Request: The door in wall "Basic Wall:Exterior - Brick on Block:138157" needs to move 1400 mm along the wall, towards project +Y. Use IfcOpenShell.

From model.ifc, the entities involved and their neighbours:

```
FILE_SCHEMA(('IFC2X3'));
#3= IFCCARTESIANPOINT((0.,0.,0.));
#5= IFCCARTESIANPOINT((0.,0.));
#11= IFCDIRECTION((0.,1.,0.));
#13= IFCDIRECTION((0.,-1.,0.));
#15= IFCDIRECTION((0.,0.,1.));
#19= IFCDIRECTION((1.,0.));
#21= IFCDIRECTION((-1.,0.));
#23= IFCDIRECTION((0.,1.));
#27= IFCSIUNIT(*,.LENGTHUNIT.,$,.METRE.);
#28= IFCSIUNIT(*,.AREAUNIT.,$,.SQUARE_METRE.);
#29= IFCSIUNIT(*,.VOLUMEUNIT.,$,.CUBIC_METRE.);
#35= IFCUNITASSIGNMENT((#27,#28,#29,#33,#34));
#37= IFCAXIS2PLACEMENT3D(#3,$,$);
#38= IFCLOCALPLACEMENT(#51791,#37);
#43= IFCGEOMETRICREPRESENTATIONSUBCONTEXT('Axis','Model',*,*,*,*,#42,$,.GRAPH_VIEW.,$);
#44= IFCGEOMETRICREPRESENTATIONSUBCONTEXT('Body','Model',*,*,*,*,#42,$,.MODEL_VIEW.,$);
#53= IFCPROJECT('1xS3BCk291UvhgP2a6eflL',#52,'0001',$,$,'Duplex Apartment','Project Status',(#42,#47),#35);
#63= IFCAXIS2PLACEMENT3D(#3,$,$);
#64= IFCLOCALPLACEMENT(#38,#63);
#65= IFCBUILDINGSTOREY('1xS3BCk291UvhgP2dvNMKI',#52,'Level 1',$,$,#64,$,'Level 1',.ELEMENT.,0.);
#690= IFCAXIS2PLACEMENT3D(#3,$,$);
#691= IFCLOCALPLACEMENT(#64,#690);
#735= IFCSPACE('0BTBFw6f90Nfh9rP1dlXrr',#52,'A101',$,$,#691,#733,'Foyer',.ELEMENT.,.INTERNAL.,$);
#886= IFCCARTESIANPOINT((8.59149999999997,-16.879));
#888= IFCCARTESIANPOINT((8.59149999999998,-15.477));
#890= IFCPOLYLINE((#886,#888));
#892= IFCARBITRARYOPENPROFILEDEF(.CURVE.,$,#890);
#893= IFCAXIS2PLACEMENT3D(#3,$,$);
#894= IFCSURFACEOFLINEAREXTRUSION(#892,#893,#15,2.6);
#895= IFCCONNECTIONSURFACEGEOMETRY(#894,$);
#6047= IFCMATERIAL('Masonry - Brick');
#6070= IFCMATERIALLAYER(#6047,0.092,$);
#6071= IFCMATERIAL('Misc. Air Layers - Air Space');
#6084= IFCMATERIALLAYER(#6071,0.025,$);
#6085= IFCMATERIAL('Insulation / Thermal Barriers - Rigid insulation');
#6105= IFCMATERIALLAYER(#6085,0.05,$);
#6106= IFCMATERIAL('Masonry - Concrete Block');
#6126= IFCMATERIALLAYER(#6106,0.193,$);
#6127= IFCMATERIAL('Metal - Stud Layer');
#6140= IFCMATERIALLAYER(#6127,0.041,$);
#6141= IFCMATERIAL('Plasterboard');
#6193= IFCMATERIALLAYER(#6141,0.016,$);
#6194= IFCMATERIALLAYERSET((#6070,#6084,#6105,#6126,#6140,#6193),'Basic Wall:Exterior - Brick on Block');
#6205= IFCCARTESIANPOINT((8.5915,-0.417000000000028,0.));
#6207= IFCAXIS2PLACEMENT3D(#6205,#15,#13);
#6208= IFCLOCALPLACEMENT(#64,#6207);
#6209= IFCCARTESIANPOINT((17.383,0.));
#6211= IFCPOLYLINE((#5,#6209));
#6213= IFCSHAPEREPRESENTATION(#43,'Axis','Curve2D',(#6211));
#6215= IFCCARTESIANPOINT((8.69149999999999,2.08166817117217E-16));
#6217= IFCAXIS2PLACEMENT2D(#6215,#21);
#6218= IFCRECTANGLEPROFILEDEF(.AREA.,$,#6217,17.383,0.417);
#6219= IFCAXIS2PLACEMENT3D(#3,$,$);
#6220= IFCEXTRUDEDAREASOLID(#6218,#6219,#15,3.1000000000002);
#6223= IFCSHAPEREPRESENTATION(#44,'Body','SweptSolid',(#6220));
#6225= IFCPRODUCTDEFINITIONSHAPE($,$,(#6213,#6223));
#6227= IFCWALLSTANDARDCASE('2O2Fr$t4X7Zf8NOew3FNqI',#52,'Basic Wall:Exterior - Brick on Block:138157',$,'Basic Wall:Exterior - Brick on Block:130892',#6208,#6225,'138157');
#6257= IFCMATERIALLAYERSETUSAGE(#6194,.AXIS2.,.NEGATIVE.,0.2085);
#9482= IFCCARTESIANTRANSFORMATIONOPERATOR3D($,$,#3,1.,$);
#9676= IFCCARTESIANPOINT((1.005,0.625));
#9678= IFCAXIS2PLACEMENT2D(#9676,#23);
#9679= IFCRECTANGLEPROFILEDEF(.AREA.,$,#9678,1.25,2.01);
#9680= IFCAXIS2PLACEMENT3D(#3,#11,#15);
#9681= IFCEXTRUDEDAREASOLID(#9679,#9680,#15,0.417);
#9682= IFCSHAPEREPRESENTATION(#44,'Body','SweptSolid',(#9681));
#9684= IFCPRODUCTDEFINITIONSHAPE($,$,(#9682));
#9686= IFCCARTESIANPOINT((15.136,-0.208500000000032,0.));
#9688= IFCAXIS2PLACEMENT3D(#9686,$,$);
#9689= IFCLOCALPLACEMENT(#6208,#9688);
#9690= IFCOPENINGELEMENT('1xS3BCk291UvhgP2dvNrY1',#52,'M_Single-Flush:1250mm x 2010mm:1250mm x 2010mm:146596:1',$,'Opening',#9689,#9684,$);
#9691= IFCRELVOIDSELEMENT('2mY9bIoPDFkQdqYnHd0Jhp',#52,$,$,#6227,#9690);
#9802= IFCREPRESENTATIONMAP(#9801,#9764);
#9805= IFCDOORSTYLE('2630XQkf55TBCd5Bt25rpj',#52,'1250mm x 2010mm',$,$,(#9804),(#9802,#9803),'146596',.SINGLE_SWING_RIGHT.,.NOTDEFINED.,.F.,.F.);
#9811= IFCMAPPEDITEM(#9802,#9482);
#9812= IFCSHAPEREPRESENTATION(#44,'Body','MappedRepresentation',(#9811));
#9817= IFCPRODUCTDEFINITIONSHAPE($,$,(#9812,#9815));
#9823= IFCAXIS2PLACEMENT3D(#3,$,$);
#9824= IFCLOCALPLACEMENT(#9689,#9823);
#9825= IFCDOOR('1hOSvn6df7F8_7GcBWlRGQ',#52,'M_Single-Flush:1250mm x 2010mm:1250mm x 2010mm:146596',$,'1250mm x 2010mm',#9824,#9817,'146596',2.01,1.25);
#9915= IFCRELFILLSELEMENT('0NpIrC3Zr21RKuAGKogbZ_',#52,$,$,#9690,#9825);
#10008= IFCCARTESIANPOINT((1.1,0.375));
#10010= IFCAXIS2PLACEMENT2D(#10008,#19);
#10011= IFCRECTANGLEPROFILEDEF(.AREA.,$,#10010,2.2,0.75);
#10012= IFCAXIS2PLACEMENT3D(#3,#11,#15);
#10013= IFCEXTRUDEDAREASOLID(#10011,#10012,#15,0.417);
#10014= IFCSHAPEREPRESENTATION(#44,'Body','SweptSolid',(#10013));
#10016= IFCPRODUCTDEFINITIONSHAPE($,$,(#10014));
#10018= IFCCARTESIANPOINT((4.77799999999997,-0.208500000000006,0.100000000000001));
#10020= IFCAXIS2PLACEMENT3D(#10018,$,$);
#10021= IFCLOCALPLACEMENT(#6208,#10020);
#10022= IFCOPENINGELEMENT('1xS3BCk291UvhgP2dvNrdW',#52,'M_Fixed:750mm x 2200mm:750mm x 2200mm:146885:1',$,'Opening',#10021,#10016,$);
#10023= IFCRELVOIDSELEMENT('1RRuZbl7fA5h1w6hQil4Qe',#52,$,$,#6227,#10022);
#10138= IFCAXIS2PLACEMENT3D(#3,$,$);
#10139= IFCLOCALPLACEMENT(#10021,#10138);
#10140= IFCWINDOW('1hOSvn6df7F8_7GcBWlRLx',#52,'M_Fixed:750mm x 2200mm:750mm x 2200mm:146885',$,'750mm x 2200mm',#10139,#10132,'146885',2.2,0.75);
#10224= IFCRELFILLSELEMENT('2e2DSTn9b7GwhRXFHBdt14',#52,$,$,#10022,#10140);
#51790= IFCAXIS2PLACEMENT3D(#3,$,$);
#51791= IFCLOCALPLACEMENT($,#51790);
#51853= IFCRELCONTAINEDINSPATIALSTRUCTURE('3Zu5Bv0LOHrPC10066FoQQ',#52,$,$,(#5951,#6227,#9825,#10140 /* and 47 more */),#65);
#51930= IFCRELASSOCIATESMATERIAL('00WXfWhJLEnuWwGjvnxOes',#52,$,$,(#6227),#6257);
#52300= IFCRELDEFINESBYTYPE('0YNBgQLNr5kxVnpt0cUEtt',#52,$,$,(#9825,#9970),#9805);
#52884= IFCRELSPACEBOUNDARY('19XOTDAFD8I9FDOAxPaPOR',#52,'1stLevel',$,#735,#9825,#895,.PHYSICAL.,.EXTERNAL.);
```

```python
import numpy as np
import ifcopenshell
import ifcopenshell.api.geometry
import ifcopenshell.util.placement

model = ifcopenshell.open("model.ifc")

door = model.by_guid("1hOSvn6df7F8_7GcBWlRGQ")
opening = door.FillsVoids[0].RelatingOpeningElement
wall = opening.VoidsElements[0].RelatingBuildingElement

wall_matrix = ifcopenshell.util.placement.get_local_placement(wall.ObjectPlacement)
shift = wall_matrix[:3, 0] * -1.4
before = ifcopenshell.util.placement.get_local_placement(door.ObjectPlacement)[:3, 3].copy()

# The door is placed relative to its opening, so it follows when the opening moves.
matrix = ifcopenshell.util.placement.get_local_placement(opening.ObjectPlacement)
matrix[:3, 3] += shift
ifcopenshell.api.geometry.edit_object_placement(
    model, product=opening, matrix=matrix, is_si=False, should_transform_children=True
)

# Space boundary surfaces are stored in each space's coordinates; move them too.
for rel in door.ProvidesBoundaries:
    if not rel.ConnectionGeometry:
        continue
    surface = rel.ConnectionGeometry.SurfaceOnRelatingElement
    space_matrix = ifcopenshell.util.placement.get_local_placement(rel.RelatingSpace.ObjectPlacement)
    point = np.array(surface.Position.Location.Coordinates) + space_matrix[:3, :3].T @ shift
    surface.Position = model.createIfcAxis2Placement3D(
        model.createIfcCartesianPoint(point.tolist()), surface.Position.Axis, surface.Position.RefDirection
    )

after = ifcopenshell.util.placement.get_local_placement(door.ObjectPlacement)[:3, 3]
print("door moved by", (after - before).round(3) + 0.0)

model.write("model_v2.ifc")
```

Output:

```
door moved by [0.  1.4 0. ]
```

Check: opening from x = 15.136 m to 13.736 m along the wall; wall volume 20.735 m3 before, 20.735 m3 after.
